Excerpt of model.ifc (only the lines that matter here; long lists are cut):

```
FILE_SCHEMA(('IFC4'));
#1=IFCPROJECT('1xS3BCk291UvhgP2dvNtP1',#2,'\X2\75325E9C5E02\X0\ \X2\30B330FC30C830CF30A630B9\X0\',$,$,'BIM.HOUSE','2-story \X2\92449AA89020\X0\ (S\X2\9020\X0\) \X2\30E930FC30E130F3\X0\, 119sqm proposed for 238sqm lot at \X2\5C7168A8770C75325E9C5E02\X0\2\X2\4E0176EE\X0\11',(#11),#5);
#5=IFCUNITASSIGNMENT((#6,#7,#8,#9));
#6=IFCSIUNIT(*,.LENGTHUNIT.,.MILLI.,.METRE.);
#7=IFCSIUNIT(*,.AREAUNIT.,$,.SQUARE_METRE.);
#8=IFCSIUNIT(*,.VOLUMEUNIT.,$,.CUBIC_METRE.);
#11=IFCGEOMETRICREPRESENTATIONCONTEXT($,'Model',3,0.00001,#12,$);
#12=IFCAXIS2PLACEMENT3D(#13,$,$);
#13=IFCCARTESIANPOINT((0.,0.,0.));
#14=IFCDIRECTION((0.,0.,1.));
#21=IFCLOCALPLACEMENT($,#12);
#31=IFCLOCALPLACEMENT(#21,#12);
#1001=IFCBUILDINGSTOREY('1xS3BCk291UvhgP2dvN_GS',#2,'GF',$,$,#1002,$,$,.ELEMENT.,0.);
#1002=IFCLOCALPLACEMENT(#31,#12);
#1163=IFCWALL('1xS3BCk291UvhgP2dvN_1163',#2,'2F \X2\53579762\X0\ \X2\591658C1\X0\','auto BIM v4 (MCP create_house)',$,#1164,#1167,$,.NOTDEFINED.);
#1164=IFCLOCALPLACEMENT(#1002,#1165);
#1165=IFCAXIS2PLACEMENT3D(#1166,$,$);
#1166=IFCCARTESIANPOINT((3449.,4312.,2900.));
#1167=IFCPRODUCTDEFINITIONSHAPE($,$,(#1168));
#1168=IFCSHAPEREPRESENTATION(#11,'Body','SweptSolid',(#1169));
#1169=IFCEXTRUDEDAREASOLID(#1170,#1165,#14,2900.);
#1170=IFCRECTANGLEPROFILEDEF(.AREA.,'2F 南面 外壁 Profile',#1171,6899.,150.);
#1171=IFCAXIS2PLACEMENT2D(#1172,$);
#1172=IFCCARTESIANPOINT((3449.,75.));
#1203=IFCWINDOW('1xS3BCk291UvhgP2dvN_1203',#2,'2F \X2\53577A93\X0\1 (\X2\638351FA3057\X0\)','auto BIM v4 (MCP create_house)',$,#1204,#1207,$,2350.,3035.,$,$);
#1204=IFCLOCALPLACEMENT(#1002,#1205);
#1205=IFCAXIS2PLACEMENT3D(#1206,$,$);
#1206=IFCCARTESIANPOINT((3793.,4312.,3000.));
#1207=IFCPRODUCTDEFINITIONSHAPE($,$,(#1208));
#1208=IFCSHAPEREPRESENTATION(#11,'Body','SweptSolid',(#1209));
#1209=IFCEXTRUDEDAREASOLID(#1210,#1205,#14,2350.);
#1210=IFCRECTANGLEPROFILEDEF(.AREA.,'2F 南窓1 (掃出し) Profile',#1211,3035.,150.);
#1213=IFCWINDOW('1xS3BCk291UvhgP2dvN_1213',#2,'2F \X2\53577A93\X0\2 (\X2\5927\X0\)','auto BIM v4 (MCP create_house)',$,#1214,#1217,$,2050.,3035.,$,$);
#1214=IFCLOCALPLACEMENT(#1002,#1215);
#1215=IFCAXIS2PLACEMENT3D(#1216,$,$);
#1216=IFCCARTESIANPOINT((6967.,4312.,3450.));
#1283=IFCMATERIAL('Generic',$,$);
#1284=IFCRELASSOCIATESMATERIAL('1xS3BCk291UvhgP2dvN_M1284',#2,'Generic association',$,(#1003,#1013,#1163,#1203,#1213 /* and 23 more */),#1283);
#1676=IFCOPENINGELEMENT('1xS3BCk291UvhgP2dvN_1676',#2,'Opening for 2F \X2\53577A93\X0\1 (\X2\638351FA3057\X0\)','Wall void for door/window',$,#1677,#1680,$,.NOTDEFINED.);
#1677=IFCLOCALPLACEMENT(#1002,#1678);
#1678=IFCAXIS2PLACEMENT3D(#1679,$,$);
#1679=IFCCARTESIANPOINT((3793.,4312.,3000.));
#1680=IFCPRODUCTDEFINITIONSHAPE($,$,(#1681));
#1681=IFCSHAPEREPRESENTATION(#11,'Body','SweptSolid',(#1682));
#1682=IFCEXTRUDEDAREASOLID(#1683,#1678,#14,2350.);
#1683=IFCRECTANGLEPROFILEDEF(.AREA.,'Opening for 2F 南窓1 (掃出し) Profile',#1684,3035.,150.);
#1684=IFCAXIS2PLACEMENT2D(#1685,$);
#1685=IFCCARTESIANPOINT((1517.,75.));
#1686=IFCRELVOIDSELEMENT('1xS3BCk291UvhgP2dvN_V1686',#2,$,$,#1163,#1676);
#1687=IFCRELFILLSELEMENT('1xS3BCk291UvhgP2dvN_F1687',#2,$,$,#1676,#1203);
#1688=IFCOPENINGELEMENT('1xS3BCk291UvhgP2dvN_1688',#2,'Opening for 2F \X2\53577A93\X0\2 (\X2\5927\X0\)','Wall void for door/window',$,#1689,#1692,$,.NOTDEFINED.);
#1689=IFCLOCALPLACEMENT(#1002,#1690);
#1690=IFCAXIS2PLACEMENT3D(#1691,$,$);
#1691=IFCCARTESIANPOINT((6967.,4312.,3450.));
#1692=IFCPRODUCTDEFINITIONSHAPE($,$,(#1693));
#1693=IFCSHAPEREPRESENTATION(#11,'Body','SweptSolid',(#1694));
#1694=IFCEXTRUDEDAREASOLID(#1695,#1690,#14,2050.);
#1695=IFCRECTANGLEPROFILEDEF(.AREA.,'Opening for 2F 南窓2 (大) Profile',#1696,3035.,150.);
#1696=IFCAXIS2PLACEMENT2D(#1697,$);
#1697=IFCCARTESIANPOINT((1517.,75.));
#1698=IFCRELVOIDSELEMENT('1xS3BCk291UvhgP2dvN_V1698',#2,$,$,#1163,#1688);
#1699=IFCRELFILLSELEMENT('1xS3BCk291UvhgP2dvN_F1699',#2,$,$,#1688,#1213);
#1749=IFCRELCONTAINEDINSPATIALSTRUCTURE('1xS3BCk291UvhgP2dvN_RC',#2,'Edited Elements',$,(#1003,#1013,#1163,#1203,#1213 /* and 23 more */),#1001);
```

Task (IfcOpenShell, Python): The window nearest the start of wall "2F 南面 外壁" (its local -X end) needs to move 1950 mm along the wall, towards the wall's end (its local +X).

```python
import ifcopenshell
import ifcopenshell.api.geometry
import ifcopenshell.util.placement
import ifcopenshell.util.unit

model = ifcopenshell.open("model.ifc")
unit_scale = ifcopenshell.util.unit.calculate_unit_scale(model)

window = model.by_id(1203)
opening = window.FillsVoids[0].RelatingOpeningElement
wall = opening.VoidsElements[0].RelatingBuildingElement

wall_matrix = ifcopenshell.util.placement.get_local_placement(wall.ObjectPlacement)
shift = wall_matrix[:3, 0] * 1.95 / unit_scale
before = ifcopenshell.util.placement.get_local_placement(window.ObjectPlacement)[:3, 3].copy()

# The window is not placed relative to its opening, so move both.
for product in (opening, window):
    matrix = ifcopenshell.util.placement.get_local_placement(product.ObjectPlacement)
    matrix[:3, 3] += shift
    ifcopenshell.api.geometry.edit_object_placement(model, product=product, matrix=matrix, is_si=False)

after = ifcopenshell.util.placement.get_local_placement(window.ObjectPlacement)[:3, 3]
print("window moved by", (after - before).round(3) + 0.0)

model.write("model_v2.ifc")
```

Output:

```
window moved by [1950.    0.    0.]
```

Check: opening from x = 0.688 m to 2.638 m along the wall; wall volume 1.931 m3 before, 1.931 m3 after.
